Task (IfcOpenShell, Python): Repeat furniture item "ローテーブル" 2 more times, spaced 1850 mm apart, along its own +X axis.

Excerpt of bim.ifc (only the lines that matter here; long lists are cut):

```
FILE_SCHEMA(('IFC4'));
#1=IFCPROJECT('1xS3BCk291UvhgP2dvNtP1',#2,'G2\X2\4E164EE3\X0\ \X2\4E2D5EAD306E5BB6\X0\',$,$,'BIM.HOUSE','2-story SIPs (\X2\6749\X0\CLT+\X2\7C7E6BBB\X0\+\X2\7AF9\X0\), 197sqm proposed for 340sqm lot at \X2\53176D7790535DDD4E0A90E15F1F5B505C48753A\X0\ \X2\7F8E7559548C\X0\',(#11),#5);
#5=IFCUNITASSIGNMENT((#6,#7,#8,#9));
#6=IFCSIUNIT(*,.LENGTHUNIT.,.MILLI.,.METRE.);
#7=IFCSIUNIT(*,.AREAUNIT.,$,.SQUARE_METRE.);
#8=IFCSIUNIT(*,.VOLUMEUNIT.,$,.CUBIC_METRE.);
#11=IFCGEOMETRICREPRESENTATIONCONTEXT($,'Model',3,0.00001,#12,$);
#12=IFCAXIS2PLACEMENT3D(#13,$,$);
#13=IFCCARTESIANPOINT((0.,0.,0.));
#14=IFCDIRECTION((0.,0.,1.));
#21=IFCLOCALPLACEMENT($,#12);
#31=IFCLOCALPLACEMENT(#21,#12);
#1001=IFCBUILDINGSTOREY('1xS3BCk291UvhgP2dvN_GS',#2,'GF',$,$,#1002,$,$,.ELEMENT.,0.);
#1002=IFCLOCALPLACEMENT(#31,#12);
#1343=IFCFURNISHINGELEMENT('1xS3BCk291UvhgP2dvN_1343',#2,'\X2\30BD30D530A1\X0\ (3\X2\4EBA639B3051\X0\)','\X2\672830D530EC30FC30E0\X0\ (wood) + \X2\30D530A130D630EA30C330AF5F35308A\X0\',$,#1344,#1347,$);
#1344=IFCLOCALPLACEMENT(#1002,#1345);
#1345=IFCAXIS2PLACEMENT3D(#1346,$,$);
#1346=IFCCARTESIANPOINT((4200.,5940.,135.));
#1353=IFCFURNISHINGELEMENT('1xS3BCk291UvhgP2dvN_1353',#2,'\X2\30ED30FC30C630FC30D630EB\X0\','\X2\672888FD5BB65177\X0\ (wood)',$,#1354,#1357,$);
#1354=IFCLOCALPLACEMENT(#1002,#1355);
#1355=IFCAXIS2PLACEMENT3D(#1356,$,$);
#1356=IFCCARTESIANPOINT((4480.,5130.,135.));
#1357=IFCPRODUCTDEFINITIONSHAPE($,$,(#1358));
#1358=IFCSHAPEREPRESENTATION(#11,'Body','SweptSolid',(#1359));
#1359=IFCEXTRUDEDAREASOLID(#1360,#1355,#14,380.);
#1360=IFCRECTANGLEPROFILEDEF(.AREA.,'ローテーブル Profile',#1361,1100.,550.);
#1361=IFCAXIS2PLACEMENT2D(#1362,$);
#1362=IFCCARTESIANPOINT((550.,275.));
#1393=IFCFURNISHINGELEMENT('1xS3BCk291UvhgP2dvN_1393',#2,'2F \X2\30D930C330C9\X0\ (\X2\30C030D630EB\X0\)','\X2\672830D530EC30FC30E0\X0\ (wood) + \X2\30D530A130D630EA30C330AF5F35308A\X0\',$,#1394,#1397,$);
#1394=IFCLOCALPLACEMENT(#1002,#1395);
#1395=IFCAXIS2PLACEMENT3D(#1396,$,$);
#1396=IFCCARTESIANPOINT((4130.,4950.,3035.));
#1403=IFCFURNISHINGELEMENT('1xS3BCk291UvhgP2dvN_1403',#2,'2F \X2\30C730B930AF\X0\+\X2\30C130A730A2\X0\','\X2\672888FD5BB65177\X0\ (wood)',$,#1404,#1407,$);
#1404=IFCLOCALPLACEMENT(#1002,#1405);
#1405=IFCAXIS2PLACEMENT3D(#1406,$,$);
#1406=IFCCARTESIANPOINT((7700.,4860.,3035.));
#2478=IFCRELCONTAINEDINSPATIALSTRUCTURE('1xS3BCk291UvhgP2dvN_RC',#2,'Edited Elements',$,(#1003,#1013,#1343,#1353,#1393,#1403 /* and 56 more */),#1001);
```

```python
import ifcopenshell
import ifcopenshell.api.geometry
import ifcopenshell.api.root
import ifcopenshell.util.element
import ifcopenshell.util.placement

model = ifcopenshell.open("bim.ifc")


def reuse_history(source, copy):
    """copy_class also copies each property set's owner history, people and application; keep the originals."""
    for rel in copy.IsDefinedBy:
        if rel.is_a("IfcRelDefinesByProperties") and (history := rel.RelatingPropertyDefinition.OwnerHistory):
            rel.RelatingPropertyDefinition.OwnerHistory = source.OwnerHistory
            ifcopenshell.util.element.remove_deep2(model, history)


source = model.by_id(1353)
base = ifcopenshell.util.placement.get_local_placement(source.ObjectPlacement)
step = base[:3, 0] * 1850.0

for i in range(1, 3):
    copy = ifcopenshell.api.root.copy_class(model, product=source)
    copy.Representation = ifcopenshell.util.element.copy_deep(
        model, source.Representation, exclude=["IfcGeometricRepresentationContext", "IfcRepresentationMap"]
    )
    reuse_history(source, copy)
    matrix = base.copy()
    matrix[:3, 3] += i * step
    print("added at", matrix[:3, 3].round(3) + 0.0)
    ifcopenshell.api.geometry.edit_object_placement(model, product=copy, matrix=matrix, is_si=False)

model.write("bim_v2.ifc")
```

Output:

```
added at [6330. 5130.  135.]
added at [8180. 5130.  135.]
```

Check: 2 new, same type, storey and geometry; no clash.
